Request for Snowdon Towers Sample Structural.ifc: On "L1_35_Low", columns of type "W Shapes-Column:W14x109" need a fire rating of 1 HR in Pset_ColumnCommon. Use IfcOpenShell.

First a look at what the model holds.

```python
import ifcopenshell
import ifcopenshell.util.element

model = ifcopenshell.open("Snowdon Towers Sample Structural.ifc")
print(model.schema)
storey = next(s for s in model.by_type("IfcBuildingStorey") if s.Name == "L1_35_Low")
columns = [e for e in ifcopenshell.util.element.get_decomposition(storey) if e.is_a("IfcColumn")]
seen = {}
for e in columns:
    element_type = ifcopenshell.util.element.get_type(e)
    key = (element_type.Name if element_type != e and element_type else None, ifcopenshell.util.element.get_pset(e, "Pset_ColumnCommon", "FireRating"))
    seen[key] = seen.get(key, 0) + 1
for (name, value), count in sorted(seen.items(), key=str):
    print(count, "x", name, "|", value)
```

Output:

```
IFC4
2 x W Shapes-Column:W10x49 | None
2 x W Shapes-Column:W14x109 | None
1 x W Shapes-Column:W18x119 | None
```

```python
import ifcopenshell
import ifcopenshell.api.pset
import ifcopenshell.util.element

model = ifcopenshell.open("Snowdon Towers Sample Structural.ifc")

storey = next(s for s in model.by_type("IfcBuildingStorey") if s.Name == "L1_35_Low")
columns = [e for e in ifcopenshell.util.element.get_decomposition(storey) if e.is_a("IfcColumn")]

count = 0
for e in columns:
    element_type = ifcopenshell.util.element.get_type(e)
    if element_type in (None, e) or element_type.Name != "W Shapes-Column:W14x109":
        continue
    # add_pset returns the element's existing set when there is one.
    pset = ifcopenshell.api.pset.add_pset(model, product=e, name="Pset_ColumnCommon")
    ifcopenshell.api.pset.edit_pset(model, pset=pset, properties={"FireRating": "1 HR"})
    count += 1

print(count, "columns updated")

model.write("Snowdon Towers Sample Structural_v2.ifc")
```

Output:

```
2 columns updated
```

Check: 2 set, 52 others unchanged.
